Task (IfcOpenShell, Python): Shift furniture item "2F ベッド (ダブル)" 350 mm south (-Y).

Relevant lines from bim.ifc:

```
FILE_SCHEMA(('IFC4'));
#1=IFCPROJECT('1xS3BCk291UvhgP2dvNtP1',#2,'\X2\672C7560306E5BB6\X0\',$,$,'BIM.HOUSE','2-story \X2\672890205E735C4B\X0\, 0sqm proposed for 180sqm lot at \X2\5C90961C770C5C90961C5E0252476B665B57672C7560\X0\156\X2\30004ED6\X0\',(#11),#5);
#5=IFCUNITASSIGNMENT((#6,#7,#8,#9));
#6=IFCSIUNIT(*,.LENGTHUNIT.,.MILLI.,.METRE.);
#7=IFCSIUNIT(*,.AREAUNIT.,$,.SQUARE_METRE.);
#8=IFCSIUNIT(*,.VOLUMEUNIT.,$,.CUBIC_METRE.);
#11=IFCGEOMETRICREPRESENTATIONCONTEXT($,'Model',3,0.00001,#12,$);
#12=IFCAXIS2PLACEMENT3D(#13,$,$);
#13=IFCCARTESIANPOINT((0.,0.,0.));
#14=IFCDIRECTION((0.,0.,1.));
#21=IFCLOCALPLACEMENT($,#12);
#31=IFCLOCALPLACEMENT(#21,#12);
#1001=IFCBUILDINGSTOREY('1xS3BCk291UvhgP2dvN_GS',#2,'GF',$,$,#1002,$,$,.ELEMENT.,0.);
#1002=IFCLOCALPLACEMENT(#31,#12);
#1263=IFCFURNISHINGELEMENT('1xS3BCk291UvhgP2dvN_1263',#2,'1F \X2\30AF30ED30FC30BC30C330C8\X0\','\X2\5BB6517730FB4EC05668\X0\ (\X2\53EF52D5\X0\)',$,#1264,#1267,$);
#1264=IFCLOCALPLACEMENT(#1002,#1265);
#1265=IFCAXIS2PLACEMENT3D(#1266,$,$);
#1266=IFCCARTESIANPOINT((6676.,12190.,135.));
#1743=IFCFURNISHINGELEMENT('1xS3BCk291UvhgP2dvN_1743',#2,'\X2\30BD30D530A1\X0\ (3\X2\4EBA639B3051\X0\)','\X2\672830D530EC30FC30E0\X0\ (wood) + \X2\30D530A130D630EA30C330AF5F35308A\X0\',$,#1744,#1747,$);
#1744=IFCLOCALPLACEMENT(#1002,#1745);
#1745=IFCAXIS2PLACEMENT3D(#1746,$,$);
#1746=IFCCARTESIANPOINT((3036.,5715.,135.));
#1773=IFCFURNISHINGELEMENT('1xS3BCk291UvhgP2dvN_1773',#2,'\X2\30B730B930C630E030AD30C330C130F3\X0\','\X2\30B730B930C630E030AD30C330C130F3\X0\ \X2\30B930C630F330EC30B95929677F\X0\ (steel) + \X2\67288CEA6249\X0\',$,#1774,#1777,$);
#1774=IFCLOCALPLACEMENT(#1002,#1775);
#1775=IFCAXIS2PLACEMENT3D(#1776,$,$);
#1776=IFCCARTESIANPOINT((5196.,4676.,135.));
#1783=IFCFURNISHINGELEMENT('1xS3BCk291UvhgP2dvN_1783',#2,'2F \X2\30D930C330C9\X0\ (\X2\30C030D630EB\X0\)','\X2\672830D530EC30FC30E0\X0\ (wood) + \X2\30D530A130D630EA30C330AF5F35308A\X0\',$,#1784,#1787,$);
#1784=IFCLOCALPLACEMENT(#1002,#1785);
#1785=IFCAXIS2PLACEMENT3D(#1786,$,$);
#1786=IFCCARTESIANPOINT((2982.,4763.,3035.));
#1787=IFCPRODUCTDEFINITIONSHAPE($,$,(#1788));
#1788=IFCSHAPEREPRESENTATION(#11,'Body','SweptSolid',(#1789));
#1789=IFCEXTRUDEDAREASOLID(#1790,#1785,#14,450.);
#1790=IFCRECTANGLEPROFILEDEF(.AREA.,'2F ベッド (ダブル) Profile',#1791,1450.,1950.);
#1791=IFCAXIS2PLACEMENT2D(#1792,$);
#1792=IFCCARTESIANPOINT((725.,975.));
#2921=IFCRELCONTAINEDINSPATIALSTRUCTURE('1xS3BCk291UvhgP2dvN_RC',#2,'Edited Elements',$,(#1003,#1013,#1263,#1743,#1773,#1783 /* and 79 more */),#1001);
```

```python
import ifcopenshell
import ifcopenshell.api.geometry
import ifcopenshell.util.placement

model = ifcopenshell.open("bim.ifc")

item = model.by_guid("1xS3BCk291UvhgP2dvN_1783")
matrix = ifcopenshell.util.placement.get_local_placement(item.ObjectPlacement)
matrix[1, 3] -= 350.0
ifcopenshell.api.geometry.edit_object_placement(model, product=item, matrix=matrix, is_si=False)

print(ifcopenshell.util.placement.get_local_placement(item.ObjectPlacement).round(3) + 0.0)

model.write("bim_updated.ifc")
```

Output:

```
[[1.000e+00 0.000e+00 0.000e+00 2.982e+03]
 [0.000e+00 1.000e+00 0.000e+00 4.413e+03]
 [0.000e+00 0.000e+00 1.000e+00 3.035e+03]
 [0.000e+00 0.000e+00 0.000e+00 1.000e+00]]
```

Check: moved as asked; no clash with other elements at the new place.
